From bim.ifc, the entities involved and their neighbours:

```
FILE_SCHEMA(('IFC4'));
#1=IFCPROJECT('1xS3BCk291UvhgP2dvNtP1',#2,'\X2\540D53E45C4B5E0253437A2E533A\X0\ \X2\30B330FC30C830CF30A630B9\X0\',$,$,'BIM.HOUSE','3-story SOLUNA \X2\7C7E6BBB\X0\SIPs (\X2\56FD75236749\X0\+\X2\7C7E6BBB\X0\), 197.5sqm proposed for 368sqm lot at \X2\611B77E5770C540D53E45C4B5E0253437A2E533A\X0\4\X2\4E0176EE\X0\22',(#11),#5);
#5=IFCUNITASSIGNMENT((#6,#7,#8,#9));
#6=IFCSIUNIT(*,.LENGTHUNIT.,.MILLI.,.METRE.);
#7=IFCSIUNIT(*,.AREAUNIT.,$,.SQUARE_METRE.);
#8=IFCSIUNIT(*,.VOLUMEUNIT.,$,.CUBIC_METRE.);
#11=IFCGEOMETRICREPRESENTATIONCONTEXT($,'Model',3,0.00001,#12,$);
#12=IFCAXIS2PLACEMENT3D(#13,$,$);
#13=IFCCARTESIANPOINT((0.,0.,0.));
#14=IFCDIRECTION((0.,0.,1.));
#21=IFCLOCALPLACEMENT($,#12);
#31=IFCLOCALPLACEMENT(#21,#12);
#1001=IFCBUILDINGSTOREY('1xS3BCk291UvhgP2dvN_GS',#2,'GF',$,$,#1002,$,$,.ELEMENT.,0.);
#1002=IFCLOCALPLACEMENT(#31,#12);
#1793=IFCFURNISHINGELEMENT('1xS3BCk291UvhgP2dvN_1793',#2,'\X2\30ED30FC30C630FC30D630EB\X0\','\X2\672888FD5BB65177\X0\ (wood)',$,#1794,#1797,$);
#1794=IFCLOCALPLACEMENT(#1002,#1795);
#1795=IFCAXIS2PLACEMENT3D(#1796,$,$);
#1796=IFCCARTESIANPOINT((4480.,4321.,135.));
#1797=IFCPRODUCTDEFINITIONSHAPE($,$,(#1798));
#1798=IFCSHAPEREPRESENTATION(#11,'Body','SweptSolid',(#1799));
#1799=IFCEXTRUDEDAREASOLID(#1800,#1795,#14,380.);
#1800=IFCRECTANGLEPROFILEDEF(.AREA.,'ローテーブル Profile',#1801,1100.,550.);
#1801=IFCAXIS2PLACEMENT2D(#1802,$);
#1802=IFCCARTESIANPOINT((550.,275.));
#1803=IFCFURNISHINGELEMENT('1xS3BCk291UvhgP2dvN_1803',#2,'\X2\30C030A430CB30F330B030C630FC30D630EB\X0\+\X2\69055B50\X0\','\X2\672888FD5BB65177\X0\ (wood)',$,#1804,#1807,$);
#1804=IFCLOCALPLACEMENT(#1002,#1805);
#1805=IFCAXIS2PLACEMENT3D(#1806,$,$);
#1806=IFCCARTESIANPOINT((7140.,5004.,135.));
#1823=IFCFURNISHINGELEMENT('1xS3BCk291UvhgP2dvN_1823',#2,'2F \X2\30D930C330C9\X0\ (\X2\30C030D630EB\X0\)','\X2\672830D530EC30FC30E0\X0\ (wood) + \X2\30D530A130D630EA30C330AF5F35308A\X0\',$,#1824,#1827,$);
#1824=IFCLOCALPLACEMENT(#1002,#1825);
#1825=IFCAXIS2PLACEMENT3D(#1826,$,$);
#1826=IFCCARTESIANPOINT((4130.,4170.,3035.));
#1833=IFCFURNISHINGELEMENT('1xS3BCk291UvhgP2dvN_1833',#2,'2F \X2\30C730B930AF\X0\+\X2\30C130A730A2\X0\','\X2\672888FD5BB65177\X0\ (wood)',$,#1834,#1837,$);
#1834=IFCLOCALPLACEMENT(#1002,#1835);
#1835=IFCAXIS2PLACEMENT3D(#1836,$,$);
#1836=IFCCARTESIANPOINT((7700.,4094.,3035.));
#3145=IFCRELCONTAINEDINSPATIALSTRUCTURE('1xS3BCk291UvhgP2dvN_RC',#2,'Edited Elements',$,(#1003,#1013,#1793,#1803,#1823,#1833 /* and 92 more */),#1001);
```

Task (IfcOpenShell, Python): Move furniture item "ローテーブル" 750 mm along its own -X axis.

```python
import ifcopenshell
import ifcopenshell.api.geometry
import ifcopenshell.util.placement
import ifcopenshell.util.unit

model = ifcopenshell.open("bim.ifc")
unit_scale = ifcopenshell.util.unit.calculate_unit_scale(model)

item = model.by_guid("1xS3BCk291UvhgP2dvN_1793")
matrix = ifcopenshell.util.placement.get_local_placement(item.ObjectPlacement)
matrix[:3, 3] -= matrix[:3, 0] * 0.75 / unit_scale
ifcopenshell.api.geometry.edit_object_placement(model, product=item, matrix=matrix, is_si=False)

print(ifcopenshell.util.placement.get_local_placement(item.ObjectPlacement).round(3) + 0.0)

model.write("bim_rev.ifc")
```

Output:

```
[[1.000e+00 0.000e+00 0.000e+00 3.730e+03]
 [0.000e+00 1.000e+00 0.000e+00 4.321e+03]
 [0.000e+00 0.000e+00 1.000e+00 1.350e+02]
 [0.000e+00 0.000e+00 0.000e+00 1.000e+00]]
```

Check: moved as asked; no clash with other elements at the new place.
